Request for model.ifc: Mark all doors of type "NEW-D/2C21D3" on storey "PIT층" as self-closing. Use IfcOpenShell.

First a look at what the model holds.

```python
import ifcopenshell
import ifcopenshell.util.element

model = ifcopenshell.open("model.ifc")
print(model.schema)
storey = next(s for s in model.by_type("IfcBuildingStorey") if s.Name == "PIT층")
doors = [e for e in ifcopenshell.util.element.get_decomposition(storey) if e.is_a("IfcDoor")]
seen = {}
for e in doors:
    element_type = ifcopenshell.util.element.get_type(e)
    key = (element_type.Name if element_type != e and element_type else None, ifcopenshell.util.element.get_pset(e, "Pset_DoorCommon", "SelfClosing"))
    seen[key] = seen.get(key, 0) + 1
for (name, value), count in sorted(seen.items(), key=str):
    print(count, "x", name, "|", value)
```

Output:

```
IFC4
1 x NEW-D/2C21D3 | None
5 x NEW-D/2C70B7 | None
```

```python
import ifcopenshell
import ifcopenshell.api.pset
import ifcopenshell.util.element

model = ifcopenshell.open("model.ifc")

storey = next(s for s in model.by_type("IfcBuildingStorey") if s.Name == "PIT층")
doors = [e for e in ifcopenshell.util.element.get_decomposition(storey) if e.is_a("IfcDoor")]

count = 0
for e in doors:
    element_type = ifcopenshell.util.element.get_type(e)
    if element_type in (None, e) or element_type.Name != "NEW-D/2C21D3":
        continue
    # add_pset returns the element's existing set when there is one.
    pset = ifcopenshell.api.pset.add_pset(model, product=e, name="Pset_DoorCommon")
    ifcopenshell.api.pset.edit_pset(model, pset=pset, properties={"SelfClosing": True})
    count += 1

print(count, "doors updated")

model.write("model_edited.ifc")
```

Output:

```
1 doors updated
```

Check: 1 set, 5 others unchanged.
